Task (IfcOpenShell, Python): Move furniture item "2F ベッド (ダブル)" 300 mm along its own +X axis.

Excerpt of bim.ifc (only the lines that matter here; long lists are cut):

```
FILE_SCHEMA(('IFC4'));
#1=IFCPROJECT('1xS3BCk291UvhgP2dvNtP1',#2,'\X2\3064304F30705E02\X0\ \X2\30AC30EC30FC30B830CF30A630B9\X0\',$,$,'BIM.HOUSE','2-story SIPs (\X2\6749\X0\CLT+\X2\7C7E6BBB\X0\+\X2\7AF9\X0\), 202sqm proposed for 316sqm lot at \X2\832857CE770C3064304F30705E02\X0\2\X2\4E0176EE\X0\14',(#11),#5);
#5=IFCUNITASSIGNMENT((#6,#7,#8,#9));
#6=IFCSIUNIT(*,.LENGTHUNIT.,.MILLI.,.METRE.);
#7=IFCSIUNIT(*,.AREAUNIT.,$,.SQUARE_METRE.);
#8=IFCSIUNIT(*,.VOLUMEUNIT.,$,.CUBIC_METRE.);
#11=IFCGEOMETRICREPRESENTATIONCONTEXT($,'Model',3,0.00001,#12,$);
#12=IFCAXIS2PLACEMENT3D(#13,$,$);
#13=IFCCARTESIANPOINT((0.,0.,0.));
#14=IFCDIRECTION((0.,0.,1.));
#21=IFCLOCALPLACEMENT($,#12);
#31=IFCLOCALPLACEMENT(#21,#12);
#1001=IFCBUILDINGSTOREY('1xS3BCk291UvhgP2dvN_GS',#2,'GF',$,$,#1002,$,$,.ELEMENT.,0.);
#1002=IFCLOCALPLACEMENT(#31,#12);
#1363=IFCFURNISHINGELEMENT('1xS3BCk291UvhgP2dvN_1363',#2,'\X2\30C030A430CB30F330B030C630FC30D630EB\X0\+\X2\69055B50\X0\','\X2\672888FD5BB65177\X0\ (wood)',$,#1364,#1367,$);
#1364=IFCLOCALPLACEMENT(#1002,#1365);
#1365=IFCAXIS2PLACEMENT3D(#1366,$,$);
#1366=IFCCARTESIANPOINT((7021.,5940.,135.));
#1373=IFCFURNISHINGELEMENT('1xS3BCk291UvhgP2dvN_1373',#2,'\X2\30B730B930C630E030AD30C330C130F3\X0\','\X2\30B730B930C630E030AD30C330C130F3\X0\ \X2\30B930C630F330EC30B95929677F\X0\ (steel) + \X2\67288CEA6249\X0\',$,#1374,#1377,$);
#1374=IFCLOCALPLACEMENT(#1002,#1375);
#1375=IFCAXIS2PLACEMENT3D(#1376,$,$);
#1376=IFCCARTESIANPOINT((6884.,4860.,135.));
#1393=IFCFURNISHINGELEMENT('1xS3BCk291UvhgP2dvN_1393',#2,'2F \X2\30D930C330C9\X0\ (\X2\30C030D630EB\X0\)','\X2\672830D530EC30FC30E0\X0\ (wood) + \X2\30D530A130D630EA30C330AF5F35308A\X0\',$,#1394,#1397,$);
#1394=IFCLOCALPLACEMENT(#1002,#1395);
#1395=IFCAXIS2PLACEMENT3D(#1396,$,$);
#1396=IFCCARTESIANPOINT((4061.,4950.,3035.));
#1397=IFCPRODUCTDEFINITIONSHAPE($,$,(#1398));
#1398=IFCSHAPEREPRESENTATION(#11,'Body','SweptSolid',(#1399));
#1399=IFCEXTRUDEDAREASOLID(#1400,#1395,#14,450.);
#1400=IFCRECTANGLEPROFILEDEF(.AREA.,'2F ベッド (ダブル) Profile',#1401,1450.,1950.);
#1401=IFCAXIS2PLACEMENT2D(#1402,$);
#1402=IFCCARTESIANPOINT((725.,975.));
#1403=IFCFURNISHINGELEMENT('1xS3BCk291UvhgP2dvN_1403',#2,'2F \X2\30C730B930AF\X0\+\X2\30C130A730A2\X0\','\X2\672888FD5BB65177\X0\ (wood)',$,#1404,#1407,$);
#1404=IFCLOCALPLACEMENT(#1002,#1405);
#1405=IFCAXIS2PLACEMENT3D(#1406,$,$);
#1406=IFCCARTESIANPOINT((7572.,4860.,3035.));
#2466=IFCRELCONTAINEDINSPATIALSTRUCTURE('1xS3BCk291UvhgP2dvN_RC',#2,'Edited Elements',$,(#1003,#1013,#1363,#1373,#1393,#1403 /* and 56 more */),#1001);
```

```python
import ifcopenshell
import ifcopenshell.api.geometry
import ifcopenshell.util.placement
import ifcopenshell.util.unit

model = ifcopenshell.open("bim.ifc")
unit_scale = ifcopenshell.util.unit.calculate_unit_scale(model)

item = model.by_guid("1xS3BCk291UvhgP2dvN_1393")
matrix = ifcopenshell.util.placement.get_local_placement(item.ObjectPlacement)
matrix[:3, 3] += matrix[:3, 0] * 0.3 / unit_scale
ifcopenshell.api.geometry.edit_object_placement(model, product=item, matrix=matrix, is_si=False)

print(ifcopenshell.util.placement.get_local_placement(item.ObjectPlacement).round(3) + 0.0)

model.write("bim-out.ifc")
```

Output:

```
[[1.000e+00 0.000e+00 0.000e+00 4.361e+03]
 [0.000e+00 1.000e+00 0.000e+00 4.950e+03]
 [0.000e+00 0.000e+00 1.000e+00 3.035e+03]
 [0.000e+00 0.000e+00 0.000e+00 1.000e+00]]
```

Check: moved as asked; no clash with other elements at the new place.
